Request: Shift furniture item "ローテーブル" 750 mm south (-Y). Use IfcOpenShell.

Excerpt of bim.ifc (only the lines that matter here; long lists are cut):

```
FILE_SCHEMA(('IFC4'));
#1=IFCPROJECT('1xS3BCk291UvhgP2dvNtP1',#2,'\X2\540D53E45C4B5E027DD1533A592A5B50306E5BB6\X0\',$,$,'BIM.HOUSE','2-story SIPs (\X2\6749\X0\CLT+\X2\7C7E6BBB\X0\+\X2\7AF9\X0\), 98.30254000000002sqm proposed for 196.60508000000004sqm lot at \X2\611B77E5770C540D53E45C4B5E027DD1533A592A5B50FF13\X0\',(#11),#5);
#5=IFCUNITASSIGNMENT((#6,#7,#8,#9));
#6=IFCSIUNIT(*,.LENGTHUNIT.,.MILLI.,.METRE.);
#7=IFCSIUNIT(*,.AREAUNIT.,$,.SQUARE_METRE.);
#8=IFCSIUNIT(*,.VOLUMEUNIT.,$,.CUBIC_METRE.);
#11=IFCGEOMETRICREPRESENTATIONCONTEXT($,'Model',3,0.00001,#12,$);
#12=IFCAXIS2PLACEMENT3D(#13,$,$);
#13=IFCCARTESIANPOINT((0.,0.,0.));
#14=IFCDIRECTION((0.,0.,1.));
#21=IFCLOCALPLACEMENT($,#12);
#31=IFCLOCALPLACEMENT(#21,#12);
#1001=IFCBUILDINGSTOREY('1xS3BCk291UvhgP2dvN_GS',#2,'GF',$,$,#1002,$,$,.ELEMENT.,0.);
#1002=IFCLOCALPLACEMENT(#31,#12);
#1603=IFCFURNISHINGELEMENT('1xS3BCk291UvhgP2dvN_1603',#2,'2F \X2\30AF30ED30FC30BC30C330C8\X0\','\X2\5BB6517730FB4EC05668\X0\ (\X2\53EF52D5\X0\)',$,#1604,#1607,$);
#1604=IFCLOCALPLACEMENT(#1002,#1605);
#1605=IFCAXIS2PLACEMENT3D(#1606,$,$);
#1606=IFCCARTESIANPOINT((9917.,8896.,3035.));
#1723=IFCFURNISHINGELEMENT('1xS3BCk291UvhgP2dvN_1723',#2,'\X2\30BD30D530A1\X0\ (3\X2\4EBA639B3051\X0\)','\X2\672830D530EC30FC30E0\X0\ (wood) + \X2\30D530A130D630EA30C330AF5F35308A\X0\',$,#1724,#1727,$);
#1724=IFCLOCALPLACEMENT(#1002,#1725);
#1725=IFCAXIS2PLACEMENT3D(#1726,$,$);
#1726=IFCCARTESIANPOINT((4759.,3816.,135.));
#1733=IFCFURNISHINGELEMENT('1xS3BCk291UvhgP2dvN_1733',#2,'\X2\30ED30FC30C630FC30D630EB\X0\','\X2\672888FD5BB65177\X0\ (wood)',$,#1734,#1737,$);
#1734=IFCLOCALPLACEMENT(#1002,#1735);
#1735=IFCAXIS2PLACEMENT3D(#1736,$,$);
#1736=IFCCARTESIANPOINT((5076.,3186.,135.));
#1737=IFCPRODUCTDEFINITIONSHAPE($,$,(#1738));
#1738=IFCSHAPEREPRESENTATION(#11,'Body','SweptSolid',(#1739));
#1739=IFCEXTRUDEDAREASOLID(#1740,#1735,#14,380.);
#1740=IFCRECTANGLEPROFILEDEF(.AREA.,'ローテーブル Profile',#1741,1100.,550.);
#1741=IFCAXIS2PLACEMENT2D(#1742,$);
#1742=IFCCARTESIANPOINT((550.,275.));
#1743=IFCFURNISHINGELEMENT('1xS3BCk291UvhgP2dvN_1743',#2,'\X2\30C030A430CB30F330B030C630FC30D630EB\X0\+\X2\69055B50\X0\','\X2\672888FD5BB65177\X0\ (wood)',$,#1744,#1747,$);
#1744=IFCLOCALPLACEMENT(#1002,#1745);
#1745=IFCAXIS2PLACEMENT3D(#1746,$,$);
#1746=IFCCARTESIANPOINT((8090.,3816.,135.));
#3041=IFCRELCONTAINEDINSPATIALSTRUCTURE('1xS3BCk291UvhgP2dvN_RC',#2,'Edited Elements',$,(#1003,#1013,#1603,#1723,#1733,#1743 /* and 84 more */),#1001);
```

```python
import ifcopenshell
import ifcopenshell.api.geometry
import ifcopenshell.util.placement

model = ifcopenshell.open("bim.ifc")

item = model.by_id(1733)
matrix = ifcopenshell.util.placement.get_local_placement(item.ObjectPlacement)
matrix[1, 3] -= 750.0
ifcopenshell.api.geometry.edit_object_placement(model, product=item, matrix=matrix, is_si=False)

print(ifcopenshell.util.placement.get_local_placement(item.ObjectPlacement).round(3) + 0.0)

model.write("bim_v2.ifc")
```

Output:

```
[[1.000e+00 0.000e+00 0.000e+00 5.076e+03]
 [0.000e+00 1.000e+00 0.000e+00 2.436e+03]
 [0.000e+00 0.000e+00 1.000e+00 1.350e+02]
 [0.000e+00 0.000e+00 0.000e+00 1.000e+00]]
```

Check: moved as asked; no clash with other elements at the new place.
